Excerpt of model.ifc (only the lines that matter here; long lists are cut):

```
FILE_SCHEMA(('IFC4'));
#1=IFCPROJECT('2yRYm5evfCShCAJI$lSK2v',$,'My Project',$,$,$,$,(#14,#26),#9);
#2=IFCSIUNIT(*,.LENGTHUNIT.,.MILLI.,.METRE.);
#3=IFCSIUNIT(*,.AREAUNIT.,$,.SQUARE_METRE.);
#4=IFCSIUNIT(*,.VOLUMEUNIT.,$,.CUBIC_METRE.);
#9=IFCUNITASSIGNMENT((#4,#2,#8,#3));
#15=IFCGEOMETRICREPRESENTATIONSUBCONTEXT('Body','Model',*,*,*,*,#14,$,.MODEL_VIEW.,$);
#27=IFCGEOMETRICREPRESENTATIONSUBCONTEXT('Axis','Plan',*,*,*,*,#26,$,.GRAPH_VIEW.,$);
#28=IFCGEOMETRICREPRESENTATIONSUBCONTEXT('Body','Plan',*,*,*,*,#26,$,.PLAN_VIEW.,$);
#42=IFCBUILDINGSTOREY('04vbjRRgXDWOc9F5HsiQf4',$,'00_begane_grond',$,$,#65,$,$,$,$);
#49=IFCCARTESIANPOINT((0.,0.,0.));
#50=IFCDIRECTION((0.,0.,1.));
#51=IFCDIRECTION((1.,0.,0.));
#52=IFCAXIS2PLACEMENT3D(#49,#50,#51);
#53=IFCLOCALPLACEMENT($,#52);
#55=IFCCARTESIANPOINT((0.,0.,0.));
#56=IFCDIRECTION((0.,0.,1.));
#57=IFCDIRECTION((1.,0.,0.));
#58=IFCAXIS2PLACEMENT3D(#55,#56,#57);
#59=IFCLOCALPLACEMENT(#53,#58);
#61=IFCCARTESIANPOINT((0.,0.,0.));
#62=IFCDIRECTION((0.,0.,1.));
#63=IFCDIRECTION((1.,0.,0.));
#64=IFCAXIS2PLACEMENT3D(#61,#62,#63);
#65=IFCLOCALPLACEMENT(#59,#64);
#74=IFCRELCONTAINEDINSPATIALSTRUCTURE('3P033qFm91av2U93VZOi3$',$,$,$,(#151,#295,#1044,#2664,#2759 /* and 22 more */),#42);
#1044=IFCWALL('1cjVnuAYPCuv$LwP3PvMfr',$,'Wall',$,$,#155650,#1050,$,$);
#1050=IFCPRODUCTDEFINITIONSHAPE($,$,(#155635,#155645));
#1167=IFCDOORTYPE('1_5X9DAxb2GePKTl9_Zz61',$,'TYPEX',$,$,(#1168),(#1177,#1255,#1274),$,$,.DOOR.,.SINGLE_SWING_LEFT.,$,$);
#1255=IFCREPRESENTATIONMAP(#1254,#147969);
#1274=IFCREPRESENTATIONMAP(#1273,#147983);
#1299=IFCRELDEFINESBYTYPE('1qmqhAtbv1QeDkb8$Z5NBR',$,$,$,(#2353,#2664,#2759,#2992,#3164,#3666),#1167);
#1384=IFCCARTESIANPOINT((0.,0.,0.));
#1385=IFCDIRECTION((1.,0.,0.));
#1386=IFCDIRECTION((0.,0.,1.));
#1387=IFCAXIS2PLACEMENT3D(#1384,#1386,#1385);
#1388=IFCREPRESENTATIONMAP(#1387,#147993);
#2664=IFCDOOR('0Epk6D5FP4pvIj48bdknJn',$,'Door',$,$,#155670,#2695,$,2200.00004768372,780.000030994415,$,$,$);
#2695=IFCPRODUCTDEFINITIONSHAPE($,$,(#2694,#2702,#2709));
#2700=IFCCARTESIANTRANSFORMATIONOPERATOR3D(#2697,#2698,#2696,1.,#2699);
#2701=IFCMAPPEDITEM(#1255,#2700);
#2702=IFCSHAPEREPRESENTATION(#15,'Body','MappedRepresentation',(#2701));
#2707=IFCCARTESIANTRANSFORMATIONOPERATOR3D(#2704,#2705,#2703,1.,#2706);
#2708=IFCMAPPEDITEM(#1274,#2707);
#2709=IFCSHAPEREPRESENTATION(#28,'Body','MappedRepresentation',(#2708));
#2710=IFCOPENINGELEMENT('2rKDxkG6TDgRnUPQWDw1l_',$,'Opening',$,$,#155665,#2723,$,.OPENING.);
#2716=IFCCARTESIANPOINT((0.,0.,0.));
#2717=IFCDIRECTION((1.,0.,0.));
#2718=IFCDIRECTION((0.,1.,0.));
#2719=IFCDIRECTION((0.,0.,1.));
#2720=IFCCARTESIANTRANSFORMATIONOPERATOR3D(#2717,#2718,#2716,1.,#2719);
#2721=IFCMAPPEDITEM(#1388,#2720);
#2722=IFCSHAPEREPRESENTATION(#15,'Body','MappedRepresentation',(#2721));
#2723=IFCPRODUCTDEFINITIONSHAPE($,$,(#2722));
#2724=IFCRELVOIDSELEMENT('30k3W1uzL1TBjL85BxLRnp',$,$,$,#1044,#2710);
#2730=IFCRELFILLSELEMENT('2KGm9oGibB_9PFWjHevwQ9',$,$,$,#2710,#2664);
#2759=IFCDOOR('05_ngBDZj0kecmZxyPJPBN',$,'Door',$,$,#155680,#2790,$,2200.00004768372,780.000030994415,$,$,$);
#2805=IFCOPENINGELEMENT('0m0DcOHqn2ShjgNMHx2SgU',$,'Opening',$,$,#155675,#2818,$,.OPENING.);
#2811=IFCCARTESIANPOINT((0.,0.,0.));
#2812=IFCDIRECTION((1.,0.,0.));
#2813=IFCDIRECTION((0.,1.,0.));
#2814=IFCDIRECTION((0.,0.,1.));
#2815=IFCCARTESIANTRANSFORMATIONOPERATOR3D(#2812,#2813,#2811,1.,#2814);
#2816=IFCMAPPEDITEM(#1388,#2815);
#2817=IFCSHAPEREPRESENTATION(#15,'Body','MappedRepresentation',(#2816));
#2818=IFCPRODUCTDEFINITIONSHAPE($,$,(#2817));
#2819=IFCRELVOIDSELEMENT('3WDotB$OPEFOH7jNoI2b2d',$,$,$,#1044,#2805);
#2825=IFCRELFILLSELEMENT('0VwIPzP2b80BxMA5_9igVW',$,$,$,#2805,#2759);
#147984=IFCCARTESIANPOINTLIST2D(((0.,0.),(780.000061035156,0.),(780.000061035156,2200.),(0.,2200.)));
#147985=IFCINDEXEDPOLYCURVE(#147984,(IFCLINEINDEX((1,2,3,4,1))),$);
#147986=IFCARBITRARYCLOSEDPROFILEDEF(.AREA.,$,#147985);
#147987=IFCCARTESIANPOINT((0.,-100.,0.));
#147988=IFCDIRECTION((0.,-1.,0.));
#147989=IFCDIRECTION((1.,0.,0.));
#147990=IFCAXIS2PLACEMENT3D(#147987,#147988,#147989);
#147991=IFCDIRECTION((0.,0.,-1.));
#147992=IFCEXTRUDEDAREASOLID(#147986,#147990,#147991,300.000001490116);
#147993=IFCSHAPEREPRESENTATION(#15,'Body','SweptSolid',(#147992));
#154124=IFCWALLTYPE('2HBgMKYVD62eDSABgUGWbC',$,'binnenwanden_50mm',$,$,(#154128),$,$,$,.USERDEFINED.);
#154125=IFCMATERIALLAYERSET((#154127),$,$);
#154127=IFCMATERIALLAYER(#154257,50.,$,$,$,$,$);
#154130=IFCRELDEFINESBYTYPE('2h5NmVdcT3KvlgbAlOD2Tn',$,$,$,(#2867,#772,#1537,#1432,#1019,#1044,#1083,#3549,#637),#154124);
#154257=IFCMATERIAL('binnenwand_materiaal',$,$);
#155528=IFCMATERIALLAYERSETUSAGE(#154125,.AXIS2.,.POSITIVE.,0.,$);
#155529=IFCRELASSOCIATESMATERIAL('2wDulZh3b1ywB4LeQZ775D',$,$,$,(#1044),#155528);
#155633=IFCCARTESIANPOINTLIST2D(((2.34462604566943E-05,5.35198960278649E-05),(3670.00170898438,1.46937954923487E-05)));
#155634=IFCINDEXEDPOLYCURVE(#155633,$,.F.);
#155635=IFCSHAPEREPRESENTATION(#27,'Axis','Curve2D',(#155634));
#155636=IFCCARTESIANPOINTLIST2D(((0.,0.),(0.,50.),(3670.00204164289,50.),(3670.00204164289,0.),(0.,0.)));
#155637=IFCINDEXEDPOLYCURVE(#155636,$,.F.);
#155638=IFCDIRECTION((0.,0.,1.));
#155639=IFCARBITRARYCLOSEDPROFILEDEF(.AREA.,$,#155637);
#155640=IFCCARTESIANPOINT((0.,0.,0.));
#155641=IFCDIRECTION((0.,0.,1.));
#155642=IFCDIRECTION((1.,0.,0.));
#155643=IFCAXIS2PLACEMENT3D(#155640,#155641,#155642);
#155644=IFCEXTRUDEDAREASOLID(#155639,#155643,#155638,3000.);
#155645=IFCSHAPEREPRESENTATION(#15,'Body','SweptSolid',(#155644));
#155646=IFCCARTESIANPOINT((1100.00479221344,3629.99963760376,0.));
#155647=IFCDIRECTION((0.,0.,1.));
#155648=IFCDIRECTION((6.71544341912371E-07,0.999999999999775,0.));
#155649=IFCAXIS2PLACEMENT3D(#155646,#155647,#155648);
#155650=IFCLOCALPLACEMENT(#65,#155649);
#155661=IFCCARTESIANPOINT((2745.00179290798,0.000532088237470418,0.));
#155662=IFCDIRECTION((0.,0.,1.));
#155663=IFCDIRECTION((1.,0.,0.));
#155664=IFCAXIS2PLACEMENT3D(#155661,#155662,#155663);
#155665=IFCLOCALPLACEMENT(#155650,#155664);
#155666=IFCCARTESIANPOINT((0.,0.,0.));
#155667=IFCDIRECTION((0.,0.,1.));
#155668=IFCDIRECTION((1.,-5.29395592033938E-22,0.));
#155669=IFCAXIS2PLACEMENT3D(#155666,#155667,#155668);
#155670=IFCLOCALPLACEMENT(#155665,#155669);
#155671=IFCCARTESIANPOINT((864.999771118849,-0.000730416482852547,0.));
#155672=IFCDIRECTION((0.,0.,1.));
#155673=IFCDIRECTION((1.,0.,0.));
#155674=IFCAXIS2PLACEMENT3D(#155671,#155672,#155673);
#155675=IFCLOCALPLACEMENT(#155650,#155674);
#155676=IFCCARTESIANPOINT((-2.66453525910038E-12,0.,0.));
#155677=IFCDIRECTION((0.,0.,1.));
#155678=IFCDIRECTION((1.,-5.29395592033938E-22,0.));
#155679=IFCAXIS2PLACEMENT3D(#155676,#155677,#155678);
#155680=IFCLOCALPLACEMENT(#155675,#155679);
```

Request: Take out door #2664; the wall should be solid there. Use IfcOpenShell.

```python
import ifcopenshell
import ifcopenshell.api.feature
import ifcopenshell.api.root
import ifcopenshell.geom
import ifcopenshell.util.shape

model = ifcopenshell.open("model.ifc")
settings = ifcopenshell.geom.settings()


def volume(element):
    """Net volume in cubic metres, openings subtracted."""
    shape = ifcopenshell.geom.create_shape(settings, element)
    return ifcopenshell.util.shape.get_volume(shape.geometry)


door = model.by_guid("0Epk6D5FP4pvIj48bdknJn")
opening = door.FillsVoids[0].RelatingOpeningElement
wall = opening.VoidsElements[0].RelatingBuildingElement
before = volume(wall)

ifcopenshell.api.root.remove_product(model, product=door)
ifcopenshell.api.feature.remove_feature(model, feature=opening)

after = volume(wall)

print(f"wall volume {before:.3f} -> {after:.3f} m3")

model.write("model_v2.ifc")
```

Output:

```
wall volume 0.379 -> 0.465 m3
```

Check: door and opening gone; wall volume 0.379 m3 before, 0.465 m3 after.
